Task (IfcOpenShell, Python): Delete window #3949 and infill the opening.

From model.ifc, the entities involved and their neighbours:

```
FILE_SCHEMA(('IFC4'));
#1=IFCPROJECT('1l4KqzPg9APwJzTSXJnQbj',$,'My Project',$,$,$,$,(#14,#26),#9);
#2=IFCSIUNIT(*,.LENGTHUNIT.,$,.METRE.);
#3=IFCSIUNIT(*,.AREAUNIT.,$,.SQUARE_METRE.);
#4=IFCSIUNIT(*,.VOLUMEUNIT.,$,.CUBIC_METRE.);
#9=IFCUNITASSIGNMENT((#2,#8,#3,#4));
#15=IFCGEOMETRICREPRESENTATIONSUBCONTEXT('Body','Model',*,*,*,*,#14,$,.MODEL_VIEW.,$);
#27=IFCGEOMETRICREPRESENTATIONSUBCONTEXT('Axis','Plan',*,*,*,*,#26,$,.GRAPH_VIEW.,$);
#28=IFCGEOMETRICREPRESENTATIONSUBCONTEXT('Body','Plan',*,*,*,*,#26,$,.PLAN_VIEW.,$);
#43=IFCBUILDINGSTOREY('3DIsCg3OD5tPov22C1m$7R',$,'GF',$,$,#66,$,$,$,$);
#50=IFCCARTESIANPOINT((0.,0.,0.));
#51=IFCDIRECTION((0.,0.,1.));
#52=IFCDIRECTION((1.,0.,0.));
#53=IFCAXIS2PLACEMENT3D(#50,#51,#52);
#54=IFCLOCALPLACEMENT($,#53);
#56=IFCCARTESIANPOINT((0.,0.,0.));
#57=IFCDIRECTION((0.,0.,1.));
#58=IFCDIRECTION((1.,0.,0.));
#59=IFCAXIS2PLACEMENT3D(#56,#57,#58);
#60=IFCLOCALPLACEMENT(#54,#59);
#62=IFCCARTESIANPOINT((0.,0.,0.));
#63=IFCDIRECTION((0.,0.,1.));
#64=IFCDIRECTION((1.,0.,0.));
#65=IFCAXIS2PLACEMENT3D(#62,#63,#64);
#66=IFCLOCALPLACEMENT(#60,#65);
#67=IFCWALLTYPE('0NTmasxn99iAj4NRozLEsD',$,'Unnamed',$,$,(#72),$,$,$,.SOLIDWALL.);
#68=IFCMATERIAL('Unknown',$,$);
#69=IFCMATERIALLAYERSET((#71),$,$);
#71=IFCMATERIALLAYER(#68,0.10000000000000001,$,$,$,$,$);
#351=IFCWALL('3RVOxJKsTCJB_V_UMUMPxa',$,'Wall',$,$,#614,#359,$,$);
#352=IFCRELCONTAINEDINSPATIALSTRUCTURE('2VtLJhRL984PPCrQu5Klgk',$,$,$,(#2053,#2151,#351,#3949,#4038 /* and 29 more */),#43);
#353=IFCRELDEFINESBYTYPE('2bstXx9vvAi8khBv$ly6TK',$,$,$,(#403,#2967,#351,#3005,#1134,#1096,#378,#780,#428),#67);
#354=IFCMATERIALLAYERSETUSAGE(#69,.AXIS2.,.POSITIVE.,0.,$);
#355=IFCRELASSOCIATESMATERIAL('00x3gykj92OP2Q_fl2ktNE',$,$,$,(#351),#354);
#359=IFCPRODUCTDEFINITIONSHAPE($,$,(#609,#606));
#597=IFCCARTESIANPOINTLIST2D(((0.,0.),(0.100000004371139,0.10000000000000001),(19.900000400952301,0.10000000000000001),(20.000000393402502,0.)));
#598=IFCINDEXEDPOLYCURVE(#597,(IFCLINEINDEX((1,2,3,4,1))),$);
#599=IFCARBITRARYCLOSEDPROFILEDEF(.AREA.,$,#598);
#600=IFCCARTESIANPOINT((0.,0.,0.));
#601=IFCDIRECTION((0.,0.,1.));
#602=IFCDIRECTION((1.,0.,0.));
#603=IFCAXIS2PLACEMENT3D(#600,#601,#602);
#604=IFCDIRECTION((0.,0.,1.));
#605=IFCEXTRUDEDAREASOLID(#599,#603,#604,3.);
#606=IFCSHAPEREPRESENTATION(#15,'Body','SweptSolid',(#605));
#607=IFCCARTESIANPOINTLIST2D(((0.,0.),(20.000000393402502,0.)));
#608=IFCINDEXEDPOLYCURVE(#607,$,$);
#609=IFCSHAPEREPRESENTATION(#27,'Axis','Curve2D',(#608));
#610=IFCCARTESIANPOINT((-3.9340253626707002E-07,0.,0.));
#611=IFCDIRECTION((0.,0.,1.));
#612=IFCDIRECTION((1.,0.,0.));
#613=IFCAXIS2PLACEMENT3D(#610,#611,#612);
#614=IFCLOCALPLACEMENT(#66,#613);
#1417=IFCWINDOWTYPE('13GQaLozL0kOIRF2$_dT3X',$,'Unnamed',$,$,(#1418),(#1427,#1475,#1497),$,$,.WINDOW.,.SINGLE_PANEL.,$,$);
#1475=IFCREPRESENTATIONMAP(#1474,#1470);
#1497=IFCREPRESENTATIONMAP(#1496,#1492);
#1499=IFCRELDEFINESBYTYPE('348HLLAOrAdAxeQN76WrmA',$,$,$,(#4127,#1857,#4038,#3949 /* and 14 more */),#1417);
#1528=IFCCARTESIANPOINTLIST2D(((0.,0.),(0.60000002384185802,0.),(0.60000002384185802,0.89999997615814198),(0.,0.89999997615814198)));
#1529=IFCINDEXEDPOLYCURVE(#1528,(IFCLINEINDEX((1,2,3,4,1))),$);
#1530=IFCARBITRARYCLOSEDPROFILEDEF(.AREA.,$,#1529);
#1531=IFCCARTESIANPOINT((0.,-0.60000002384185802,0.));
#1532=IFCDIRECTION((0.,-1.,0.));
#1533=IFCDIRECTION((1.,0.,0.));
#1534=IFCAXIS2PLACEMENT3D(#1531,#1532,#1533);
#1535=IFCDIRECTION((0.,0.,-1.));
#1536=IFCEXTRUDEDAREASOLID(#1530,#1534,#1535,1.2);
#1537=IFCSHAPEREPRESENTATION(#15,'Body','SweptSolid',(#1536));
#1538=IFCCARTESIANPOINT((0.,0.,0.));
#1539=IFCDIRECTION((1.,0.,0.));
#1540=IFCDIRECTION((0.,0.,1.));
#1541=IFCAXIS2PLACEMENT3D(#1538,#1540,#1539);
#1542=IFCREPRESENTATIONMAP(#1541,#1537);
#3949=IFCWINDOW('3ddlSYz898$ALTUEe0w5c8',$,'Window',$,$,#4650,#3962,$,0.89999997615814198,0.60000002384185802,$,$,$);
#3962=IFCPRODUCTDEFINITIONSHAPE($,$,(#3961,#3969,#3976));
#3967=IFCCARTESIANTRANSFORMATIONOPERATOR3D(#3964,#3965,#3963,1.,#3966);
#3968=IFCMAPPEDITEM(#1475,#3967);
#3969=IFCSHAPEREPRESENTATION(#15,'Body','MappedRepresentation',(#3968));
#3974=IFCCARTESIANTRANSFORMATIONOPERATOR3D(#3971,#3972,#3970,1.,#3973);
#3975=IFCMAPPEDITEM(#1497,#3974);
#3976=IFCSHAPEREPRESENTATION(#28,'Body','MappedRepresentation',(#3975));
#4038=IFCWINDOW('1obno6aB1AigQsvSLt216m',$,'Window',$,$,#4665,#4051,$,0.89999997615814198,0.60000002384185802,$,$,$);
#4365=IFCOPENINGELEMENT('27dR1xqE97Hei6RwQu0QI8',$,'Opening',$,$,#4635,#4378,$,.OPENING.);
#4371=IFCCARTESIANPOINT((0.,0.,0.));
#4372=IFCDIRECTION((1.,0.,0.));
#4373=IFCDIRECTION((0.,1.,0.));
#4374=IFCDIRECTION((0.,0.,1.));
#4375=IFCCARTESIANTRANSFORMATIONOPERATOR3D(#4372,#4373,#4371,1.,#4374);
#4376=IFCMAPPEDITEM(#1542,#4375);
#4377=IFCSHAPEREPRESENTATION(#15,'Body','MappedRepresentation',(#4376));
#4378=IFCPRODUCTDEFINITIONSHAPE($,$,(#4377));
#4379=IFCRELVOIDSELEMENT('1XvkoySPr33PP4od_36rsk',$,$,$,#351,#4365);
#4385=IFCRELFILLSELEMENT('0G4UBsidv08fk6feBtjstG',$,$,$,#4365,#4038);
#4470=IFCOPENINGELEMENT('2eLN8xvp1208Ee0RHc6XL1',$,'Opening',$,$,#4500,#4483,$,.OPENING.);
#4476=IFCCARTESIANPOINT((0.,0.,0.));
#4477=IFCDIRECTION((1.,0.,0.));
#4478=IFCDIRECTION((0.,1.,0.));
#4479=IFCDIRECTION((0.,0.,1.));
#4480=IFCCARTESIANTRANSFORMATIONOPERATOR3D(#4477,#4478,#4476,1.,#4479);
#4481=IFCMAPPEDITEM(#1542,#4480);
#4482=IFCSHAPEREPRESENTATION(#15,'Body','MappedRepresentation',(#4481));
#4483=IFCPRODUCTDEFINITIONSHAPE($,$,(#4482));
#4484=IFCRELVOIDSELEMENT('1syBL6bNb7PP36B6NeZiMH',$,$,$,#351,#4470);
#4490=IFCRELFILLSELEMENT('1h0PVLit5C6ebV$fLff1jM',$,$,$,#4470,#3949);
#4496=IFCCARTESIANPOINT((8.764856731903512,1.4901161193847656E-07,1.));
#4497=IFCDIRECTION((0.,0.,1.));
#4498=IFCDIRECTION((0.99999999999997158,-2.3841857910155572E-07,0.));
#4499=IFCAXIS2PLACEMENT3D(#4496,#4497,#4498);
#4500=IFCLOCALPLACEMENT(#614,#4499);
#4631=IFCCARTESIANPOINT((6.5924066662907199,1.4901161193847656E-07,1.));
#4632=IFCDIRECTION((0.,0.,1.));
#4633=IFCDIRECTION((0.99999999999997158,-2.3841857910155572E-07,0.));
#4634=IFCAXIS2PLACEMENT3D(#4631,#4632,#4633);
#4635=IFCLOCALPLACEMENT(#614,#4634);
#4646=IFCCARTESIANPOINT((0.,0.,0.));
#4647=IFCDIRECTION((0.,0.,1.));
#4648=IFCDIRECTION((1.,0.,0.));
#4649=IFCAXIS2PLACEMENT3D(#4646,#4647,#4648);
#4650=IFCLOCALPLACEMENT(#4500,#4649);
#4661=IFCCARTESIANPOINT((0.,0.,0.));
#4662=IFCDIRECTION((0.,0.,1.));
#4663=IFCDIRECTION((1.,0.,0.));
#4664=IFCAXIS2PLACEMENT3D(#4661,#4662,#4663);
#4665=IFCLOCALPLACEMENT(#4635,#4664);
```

```python
import ifcopenshell
import ifcopenshell.api.feature
import ifcopenshell.api.root
import ifcopenshell.geom
import ifcopenshell.util.shape

model = ifcopenshell.open("model.ifc")
settings = ifcopenshell.geom.settings()


def volume(element):
    """Net volume in cubic metres, openings subtracted."""
    shape = ifcopenshell.geom.create_shape(settings, element)
    return ifcopenshell.util.shape.get_volume(shape.geometry)


window = model.by_guid("3ddlSYz898$ALTUEe0w5c8")
opening = window.FillsVoids[0].RelatingOpeningElement
wall = opening.VoidsElements[0].RelatingBuildingElement
before = volume(wall)

ifcopenshell.api.root.remove_product(model, product=window)
ifcopenshell.api.feature.remove_feature(model, feature=opening)

after = volume(wall)

print(f"wall volume {before:.3f} -> {after:.3f} m3")

model.write("model_v2.ifc")
```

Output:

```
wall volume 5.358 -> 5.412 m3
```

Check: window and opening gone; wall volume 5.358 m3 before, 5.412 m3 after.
